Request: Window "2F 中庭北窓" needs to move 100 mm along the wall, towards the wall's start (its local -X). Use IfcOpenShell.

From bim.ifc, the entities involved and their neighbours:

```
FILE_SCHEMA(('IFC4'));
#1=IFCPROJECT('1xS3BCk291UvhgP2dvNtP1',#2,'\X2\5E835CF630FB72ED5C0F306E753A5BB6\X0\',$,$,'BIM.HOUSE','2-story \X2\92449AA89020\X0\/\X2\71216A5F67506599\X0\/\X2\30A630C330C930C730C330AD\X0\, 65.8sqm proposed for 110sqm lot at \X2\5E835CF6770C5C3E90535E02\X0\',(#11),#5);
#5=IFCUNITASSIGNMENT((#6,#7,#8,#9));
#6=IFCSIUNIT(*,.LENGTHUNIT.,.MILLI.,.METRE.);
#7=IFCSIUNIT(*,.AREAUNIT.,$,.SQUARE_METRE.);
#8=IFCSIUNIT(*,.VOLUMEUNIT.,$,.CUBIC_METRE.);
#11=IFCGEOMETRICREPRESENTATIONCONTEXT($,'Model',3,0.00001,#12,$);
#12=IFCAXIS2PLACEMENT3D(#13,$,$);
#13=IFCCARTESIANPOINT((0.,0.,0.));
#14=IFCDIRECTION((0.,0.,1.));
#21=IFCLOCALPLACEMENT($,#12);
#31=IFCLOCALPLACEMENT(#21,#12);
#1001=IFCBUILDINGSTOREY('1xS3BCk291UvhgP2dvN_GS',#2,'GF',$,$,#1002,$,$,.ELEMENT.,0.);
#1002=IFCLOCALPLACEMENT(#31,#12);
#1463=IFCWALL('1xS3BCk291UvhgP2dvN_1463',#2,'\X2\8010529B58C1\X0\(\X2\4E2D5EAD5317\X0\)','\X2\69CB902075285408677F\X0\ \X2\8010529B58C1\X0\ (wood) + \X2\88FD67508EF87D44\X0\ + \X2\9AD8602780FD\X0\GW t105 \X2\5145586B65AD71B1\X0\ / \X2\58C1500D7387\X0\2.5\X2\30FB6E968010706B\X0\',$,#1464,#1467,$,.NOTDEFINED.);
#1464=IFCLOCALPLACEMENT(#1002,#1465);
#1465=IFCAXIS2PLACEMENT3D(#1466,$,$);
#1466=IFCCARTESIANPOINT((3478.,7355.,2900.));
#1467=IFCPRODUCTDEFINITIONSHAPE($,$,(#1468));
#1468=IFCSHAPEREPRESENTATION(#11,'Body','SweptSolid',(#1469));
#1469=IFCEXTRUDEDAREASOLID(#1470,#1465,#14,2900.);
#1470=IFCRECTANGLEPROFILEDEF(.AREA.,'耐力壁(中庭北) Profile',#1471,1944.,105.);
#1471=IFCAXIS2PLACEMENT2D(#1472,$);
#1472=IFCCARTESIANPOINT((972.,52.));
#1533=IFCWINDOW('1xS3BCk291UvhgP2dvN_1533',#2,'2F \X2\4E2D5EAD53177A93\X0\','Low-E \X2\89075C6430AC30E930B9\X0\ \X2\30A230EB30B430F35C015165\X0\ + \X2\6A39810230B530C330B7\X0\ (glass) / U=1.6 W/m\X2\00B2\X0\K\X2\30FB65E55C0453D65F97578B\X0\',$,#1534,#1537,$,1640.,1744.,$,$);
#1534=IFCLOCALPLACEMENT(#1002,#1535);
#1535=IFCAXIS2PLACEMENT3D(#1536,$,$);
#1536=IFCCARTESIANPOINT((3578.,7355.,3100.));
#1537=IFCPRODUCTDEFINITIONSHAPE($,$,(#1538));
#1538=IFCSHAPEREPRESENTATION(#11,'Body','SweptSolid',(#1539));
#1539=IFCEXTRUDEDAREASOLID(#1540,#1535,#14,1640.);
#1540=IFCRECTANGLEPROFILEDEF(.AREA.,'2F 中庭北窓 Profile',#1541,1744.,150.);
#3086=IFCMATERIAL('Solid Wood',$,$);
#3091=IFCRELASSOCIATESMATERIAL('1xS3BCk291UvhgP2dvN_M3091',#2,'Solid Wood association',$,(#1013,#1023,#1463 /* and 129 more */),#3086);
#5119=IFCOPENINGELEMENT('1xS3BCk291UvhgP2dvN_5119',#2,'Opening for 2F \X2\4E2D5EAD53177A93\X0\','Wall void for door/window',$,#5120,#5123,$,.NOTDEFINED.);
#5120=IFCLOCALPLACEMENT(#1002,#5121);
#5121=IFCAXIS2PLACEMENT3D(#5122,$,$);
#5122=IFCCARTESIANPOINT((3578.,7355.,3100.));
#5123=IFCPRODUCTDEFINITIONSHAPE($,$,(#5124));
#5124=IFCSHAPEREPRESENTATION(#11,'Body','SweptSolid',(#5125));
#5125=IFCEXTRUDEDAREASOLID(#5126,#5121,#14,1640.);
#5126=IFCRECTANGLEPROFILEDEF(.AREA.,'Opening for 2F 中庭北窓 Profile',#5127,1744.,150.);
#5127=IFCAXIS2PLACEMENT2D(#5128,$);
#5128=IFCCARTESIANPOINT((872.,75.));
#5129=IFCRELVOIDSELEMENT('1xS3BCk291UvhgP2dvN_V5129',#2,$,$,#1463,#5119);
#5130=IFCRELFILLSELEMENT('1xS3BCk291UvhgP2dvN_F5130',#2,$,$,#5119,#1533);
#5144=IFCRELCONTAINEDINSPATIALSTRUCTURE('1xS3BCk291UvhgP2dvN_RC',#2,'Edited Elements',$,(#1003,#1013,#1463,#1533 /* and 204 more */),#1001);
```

```python
import ifcopenshell
import ifcopenshell.api.geometry
import ifcopenshell.util.placement
import ifcopenshell.util.unit

model = ifcopenshell.open("bim.ifc")
unit_scale = ifcopenshell.util.unit.calculate_unit_scale(model)

window = model.by_guid("1xS3BCk291UvhgP2dvN_1533")
opening = window.FillsVoids[0].RelatingOpeningElement
wall = opening.VoidsElements[0].RelatingBuildingElement

wall_matrix = ifcopenshell.util.placement.get_local_placement(wall.ObjectPlacement)
shift = wall_matrix[:3, 0] * -0.1 / unit_scale
before = ifcopenshell.util.placement.get_local_placement(window.ObjectPlacement)[:3, 3].copy()

# The window is not placed relative to its opening, so move both.
for product in (opening, window):
    matrix = ifcopenshell.util.placement.get_local_placement(product.ObjectPlacement)
    matrix[:3, 3] += shift
    ifcopenshell.api.geometry.edit_object_placement(model, product=product, matrix=matrix, is_si=False)

after = ifcopenshell.util.placement.get_local_placement(window.ObjectPlacement)[:3, 3]
print("window moved by", (after - before).round(3) + 0.0)

model.write("bim_v2.ifc")
```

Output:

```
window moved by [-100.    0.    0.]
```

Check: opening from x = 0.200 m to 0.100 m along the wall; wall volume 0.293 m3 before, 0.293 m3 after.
